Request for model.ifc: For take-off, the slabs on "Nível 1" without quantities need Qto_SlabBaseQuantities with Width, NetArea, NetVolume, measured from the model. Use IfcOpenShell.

First a look at what the model holds.

```python
import ifcopenshell
import ifcopenshell.util.element
import ifcopenshell.util.unit

model = ifcopenshell.open("model.ifc")
print(model.schema)
for unit_type in ("LENGTHUNIT", "AREAUNIT", "VOLUMEUNIT"):
    print(unit_type, ifcopenshell.util.unit.calculate_unit_scale(model, unit_type))
storey = next(s for s in model.by_type("IfcBuildingStorey") if s.Name == "Nível 1")
slabs = [e for e in ifcopenshell.util.element.get_decomposition(storey) if e.is_a("IfcSlab")]
for e in sorted(slabs, key=lambda e: e.id()):
    print(e.id(), e.is_a(), e.Name, list(ifcopenshell.util.element.get_psets(e, qtos_only=True)), sep=" | ")
```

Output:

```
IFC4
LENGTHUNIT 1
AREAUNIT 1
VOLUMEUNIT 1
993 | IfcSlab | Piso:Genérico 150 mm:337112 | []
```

```python
import ifcopenshell
import ifcopenshell.api.pset
import ifcopenshell.geom
import ifcopenshell.util.element
import ifcopenshell.util.shape
import ifcopenshell.util.unit

model = ifcopenshell.open("model.ifc")
unit_scale = ifcopenshell.util.unit.calculate_unit_scale(model)
area_scale = ifcopenshell.util.unit.calculate_unit_scale(model, "AREAUNIT")
volume_scale = ifcopenshell.util.unit.calculate_unit_scale(model, "VOLUMEUNIT")
settings = ifcopenshell.geom.settings()

storey = next(s for s in model.by_type("IfcBuildingStorey") if s.Name == "Nível 1")
slabs = [e for e in ifcopenshell.util.element.get_decomposition(storey) if e.is_a("IfcSlab")]

for e in sorted(slabs, key=lambda e: e.id()):
    if ifcopenshell.util.element.get_psets(e, qtos_only=True, should_inherit=False):
        continue
    # Geometry comes back in metres, in the element's own axes.
    shape = ifcopenshell.geom.create_shape(settings, e)
    values = {
        "Width": ifcopenshell.util.shape.get_z(shape.geometry) / unit_scale,
        "NetArea": ifcopenshell.util.shape.get_footprint_area(shape.geometry) / area_scale,
        "NetVolume": ifcopenshell.util.shape.get_volume(shape.geometry) / volume_scale,
    }
    qto = ifcopenshell.api.pset.add_qto(model, product=e, name="Qto_SlabBaseQuantities")
    ifcopenshell.api.pset.edit_qto(model, qto=qto, properties=values)
    print(e.id(), {k: round(v, 3) for k, v in values.items()})

model.write("model_v2.ifc")
```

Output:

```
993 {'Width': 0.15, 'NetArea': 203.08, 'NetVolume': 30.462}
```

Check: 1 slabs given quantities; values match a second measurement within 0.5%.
